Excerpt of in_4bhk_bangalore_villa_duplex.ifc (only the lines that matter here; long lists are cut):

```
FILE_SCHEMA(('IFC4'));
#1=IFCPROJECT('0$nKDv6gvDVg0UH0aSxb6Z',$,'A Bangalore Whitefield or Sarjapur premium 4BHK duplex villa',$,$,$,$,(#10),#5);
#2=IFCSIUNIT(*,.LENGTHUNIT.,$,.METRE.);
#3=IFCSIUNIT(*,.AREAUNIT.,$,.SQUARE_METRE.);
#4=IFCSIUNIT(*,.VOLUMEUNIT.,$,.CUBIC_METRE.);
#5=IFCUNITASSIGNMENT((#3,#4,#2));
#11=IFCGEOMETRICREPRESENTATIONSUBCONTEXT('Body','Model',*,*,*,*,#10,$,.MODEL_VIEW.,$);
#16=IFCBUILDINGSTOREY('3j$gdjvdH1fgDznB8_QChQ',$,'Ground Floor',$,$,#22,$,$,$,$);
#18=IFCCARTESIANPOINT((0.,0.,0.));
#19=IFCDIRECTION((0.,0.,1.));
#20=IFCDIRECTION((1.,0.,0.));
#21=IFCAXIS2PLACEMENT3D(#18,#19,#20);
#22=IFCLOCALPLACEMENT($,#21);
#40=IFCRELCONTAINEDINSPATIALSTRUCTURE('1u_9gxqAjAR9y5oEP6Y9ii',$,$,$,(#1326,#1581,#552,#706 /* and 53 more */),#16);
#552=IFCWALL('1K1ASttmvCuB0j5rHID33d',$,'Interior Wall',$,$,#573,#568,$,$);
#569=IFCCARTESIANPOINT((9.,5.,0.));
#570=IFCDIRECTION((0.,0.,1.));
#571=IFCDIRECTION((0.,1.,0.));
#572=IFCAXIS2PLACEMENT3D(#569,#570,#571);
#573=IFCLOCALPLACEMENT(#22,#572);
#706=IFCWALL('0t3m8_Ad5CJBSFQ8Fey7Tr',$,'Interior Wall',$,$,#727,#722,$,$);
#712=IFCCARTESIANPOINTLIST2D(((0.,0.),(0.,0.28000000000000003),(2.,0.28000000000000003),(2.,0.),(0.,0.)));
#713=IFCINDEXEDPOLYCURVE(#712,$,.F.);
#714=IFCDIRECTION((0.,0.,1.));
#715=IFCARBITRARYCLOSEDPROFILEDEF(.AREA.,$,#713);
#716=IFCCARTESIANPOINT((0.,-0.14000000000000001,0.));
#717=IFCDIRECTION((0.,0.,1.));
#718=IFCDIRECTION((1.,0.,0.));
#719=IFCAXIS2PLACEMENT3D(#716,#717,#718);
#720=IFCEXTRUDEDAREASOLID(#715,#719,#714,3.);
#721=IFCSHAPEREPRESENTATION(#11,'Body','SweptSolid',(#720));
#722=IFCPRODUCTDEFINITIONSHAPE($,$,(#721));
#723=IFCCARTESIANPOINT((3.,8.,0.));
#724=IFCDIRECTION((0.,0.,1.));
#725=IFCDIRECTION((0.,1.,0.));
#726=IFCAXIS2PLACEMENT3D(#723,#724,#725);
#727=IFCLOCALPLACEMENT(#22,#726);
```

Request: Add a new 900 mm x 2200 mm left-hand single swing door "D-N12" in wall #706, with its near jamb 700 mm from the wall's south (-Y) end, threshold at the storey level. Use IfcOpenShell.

```python
import numpy as np
import ifcopenshell
import ifcopenshell.api.feature
import ifcopenshell.api.geometry
import ifcopenshell.api.root
import ifcopenshell.api.spatial
import ifcopenshell.geom
import ifcopenshell.util.element
import ifcopenshell.util.placement
import ifcopenshell.util.representation
import ifcopenshell.util.shape
import ifcopenshell.util.unit

model = ifcopenshell.open("in_4bhk_bangalore_villa_duplex.ifc")
unit_scale = ifcopenshell.util.unit.calculate_unit_scale(model)
settings = ifcopenshell.geom.settings()


def volume(element):
    """Net volume in cubic metres, openings subtracted."""
    shape = ifcopenshell.geom.create_shape(settings, element)
    return ifcopenshell.util.shape.get_volume(shape.geometry)


wall = model.by_guid("0t3m8_Ad5CJBSFQ8Fey7Tr")
storey = ifcopenshell.util.element.get_container(wall, ifc_class="IfcBuildingStorey")
context = ifcopenshell.util.representation.get_context(model, "Model", "Body", "MODEL_VIEW")
before = volume(wall)

width, height, from_end, sill = 0.9, 2.2, 0.7, 0.0  # metres

# The wall runs along its own X axis, and the end named is its -X end.
wall_shape = ifcopenshell.geom.create_shape(settings, wall)
x, y, z = ifcopenshell.util.shape.get_vertices(wall_shape.geometry).T
start = x.min() + from_end
face, thickness = float(y.min()), float(y.max() - y.min())
wall_matrix = ifcopenshell.util.placement.get_local_placement(wall.ObjectPlacement)
level = ifcopenshell.util.placement.get_local_placement(storey.ObjectPlacement)[2, 3]


def in_wall(x, y):
    """Placement at x, y metres in the wall's axes, at sill height."""
    matrix = wall_matrix.copy()
    matrix[:, 3] = wall_matrix @ np.array([x / unit_scale, y / unit_scale, 0.0, 1.0])
    matrix[2, 3] = level + sill / unit_scale
    return matrix


# Opening: a box that overshoots both wall faces by 50 mm.
opening = ifcopenshell.api.root.create_entity(model, ifc_class="IfcOpeningElement", predefined_type="OPENING")
box = ifcopenshell.api.geometry.add_wall_representation(
    model, context=context, length=width, height=height, thickness=thickness + 0.1
)
ifcopenshell.api.geometry.assign_representation(model, product=opening, representation=box)
ifcopenshell.api.geometry.edit_object_placement(model, product=opening, matrix=in_wall(start, face - 0.05), is_si=False)
ifcopenshell.api.feature.add_feature(model, feature=opening, element=wall)

door = ifcopenshell.api.root.create_entity(model, ifc_class="IfcDoor", name="D-N12", predefined_type="DOOR")
door.OverallWidth, door.OverallHeight = width / unit_scale, height / unit_scale
door.OperationType = "SINGLE_SWING_LEFT"
body = ifcopenshell.api.geometry.add_door_representation(
    model,
    context=context,
    overall_width=door.OverallWidth,
    overall_height=door.OverallHeight,
    operation_type="SINGLE_SWING_LEFT",
    lining_properties={"LiningDepth": thickness / unit_scale, "ThresholdDepth": thickness / unit_scale},
)
ifcopenshell.api.geometry.assign_representation(model, product=door, representation=body)
ifcopenshell.api.spatial.assign_container(model, products=[door], relating_structure=storey)
ifcopenshell.api.feature.add_filling(model, opening=opening, element=door)

# The lining spans the wall, so the door starts at the wall face.
ifcopenshell.api.geometry.edit_object_placement(model, product=door, matrix=in_wall(start, face), is_si=False)

after = volume(wall)

print(f"wall volume {before:.3f} -> {after:.3f} m3")

model.write("in_4bhk_bangalore_villa_duplex_edited.ifc")
```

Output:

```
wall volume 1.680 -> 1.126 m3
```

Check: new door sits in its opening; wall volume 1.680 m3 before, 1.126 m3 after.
